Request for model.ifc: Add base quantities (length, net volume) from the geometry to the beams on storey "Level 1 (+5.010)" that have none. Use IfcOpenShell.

First a look at what the model holds.

```python
import ifcopenshell
import ifcopenshell.util.element
import ifcopenshell.util.unit

model = ifcopenshell.open("model.ifc")
print(model.schema)
for unit_type in ("LENGTHUNIT", "AREAUNIT", "VOLUMEUNIT"):
    print(unit_type, ifcopenshell.util.unit.calculate_unit_scale(model, unit_type))
storey = next(s for s in model.by_type("IfcBuildingStorey") if s.Name == "Level 1 (+5.010)")
beams = [e for e in ifcopenshell.util.element.get_decomposition(storey) if e.is_a("IfcBeam")]
for e in sorted(beams, key=lambda e: e.id()):
    print(e.id(), e.is_a(), e.Name, list(ifcopenshell.util.element.get_psets(e, qtos_only=True)), sep=" | ")
```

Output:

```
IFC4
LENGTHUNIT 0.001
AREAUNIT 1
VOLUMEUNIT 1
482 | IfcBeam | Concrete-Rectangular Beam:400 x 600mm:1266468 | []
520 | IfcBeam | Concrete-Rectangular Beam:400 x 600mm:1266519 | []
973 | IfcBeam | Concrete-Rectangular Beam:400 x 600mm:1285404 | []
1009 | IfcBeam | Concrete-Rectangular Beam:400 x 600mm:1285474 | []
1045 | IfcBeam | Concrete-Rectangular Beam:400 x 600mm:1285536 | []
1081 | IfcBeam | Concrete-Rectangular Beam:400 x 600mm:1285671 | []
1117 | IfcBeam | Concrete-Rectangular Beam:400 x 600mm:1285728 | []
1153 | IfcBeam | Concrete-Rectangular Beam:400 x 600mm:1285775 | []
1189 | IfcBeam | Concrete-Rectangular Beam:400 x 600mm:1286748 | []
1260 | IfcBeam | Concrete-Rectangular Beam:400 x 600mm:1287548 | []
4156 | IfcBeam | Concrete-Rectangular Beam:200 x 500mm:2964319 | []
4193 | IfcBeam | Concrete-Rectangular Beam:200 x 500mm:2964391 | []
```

```python
import ifcopenshell
import ifcopenshell.api.pset
import ifcopenshell.geom
import ifcopenshell.util.element
import ifcopenshell.util.shape
import ifcopenshell.util.unit

model = ifcopenshell.open("model.ifc")
unit_scale = ifcopenshell.util.unit.calculate_unit_scale(model)
volume_scale = ifcopenshell.util.unit.calculate_unit_scale(model, "VOLUMEUNIT")
settings = ifcopenshell.geom.settings()

storey = next(s for s in model.by_type("IfcBuildingStorey") if s.Name == "Level 1 (+5.010)")
beams = [e for e in ifcopenshell.util.element.get_decomposition(storey) if e.is_a("IfcBeam")]

for e in sorted(beams, key=lambda e: e.id()):
    if ifcopenshell.util.element.get_psets(e, qtos_only=True, should_inherit=False):
        continue
    # Geometry comes back in metres, in the element's own axes.
    shape = ifcopenshell.geom.create_shape(settings, e)
    values = {
        "Length": ifcopenshell.util.shape.get_max_xyz(shape.geometry) / unit_scale,
        "NetVolume": ifcopenshell.util.shape.get_volume(shape.geometry) / volume_scale,
    }
    qto = ifcopenshell.api.pset.add_qto(model, product=e, name="Qto_BeamBaseQuantities")
    ifcopenshell.api.pset.edit_qto(model, qto=qto, properties=values)
    print(e.id(), {k: round(v, 3) for k, v in values.items()})

model.write("model-out.ifc")
```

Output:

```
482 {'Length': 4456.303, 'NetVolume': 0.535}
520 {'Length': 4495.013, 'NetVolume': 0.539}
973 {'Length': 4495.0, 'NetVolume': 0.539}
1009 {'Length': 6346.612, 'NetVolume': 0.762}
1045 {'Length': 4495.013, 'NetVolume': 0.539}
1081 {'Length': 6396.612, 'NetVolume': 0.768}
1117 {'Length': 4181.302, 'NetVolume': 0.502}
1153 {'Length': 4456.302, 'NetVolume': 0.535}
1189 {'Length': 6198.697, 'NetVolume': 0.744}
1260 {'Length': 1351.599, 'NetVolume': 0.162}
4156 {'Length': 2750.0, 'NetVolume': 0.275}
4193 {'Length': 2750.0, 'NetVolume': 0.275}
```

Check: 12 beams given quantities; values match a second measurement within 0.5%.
